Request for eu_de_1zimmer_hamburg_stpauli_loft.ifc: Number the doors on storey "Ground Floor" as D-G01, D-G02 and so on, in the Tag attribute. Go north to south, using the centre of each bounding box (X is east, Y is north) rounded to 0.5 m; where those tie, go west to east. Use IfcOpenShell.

First a look at what the model holds.

```python
import ifcopenshell
import ifcopenshell.util.element
import ifcopenshell.util.placement

model = ifcopenshell.open("eu_de_1zimmer_hamburg_stpauli_loft.ifc")
print(model.schema)
storey = next(s for s in model.by_type("IfcBuildingStorey") if s.Name == "Ground Floor")
doors = [e for e in ifcopenshell.util.element.get_decomposition(storey) if e.is_a("IfcDoor")]
for e in sorted(doors, key=lambda e: e.id()):
    origin = ifcopenshell.util.placement.get_local_placement(e.ObjectPlacement)[:3, 3]
    print(e.id(), e.Tag, e.Name, origin.round(2) + 0.0, sep=" | ")
```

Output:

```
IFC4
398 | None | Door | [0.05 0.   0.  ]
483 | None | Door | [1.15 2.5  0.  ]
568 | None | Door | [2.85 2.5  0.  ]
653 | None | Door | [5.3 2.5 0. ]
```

```python
import ifcopenshell
import ifcopenshell.geom
import ifcopenshell.util.element
import ifcopenshell.util.shape

model = ifcopenshell.open("eu_de_1zimmer_hamburg_stpauli_loft.ifc")
settings = ifcopenshell.geom.settings()
settings.set("use-world-coords", True)


def centre(element):
    shape = ifcopenshell.geom.create_shape(settings, element)
    return ifcopenshell.util.shape.get_bbox_centroid(shape.geometry)


storey = next(s for s in model.by_type("IfcBuildingStorey") if s.Name == "Ground Floor")
doors = [e for e in ifcopenshell.util.element.get_decomposition(storey) if e.is_a("IfcDoor")]

# Insertion points can sit at a corner or the storey origin, so sort by the geometry (in metres).
centres = {e: centre(e) for e in doors}
doors.sort(key=lambda e: (-round(centres[e][1] / 0.5), centres[e][0]))

for i, e in enumerate(doors, start=1):
    number = f"D-G{i:02d}"
    e.Tag = number
    print(e.id(), number)

model.write("eu_de_1zimmer_hamburg_stpauli_loft_v2.ifc")
```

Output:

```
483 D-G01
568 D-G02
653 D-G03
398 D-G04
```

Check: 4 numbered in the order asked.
